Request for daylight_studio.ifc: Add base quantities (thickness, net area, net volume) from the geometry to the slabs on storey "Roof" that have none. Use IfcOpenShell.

First a look at what the model holds.

```python
import ifcopenshell
import ifcopenshell.util.element
import ifcopenshell.util.unit

model = ifcopenshell.open("daylight_studio.ifc")
print(model.schema)
for unit_type in ("LENGTHUNIT", "AREAUNIT", "VOLUMEUNIT"):
    print(unit_type, ifcopenshell.util.unit.calculate_unit_scale(model, unit_type))
storey = next(s for s in model.by_type("IfcBuildingStorey") if s.Name == "Roof")
slabs = [e for e in ifcopenshell.util.element.get_decomposition(storey) if e.is_a("IfcSlab")]
for e in sorted(slabs, key=lambda e: e.id()):
    print(e.id(), e.is_a(), e.Name, list(ifcopenshell.util.element.get_psets(e, qtos_only=True)), sep=" | ")
```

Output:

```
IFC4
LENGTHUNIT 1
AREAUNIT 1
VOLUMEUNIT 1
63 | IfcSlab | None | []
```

```python
import ifcopenshell
import ifcopenshell.api.pset
import ifcopenshell.geom
import ifcopenshell.util.element
import ifcopenshell.util.shape
import ifcopenshell.util.unit

model = ifcopenshell.open("daylight_studio.ifc")
unit_scale = ifcopenshell.util.unit.calculate_unit_scale(model)
area_scale = ifcopenshell.util.unit.calculate_unit_scale(model, "AREAUNIT")
volume_scale = ifcopenshell.util.unit.calculate_unit_scale(model, "VOLUMEUNIT")
settings = ifcopenshell.geom.settings()

storey = next(s for s in model.by_type("IfcBuildingStorey") if s.Name == "Roof")
slabs = [e for e in ifcopenshell.util.element.get_decomposition(storey) if e.is_a("IfcSlab")]

for e in sorted(slabs, key=lambda e: e.id()):
    if ifcopenshell.util.element.get_psets(e, qtos_only=True, should_inherit=False):
        continue
    # Geometry comes back in metres, in the element's own axes.
    shape = ifcopenshell.geom.create_shape(settings, e)
    values = {
        "Width": ifcopenshell.util.shape.get_z(shape.geometry) / unit_scale,
        "NetArea": ifcopenshell.util.shape.get_footprint_area(shape.geometry) / area_scale,
        "NetVolume": ifcopenshell.util.shape.get_volume(shape.geometry) / volume_scale,
    }
    qto = ifcopenshell.api.pset.add_qto(model, product=e, name="Qto_SlabBaseQuantities")
    ifcopenshell.api.pset.edit_qto(model, qto=qto, properties=values)
    print(e.id(), {k: round(v, 3) for k, v in values.items()})

model.write("daylight_studio_updated.ifc")
```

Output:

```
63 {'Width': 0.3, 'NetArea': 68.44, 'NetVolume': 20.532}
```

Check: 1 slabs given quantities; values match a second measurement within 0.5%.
